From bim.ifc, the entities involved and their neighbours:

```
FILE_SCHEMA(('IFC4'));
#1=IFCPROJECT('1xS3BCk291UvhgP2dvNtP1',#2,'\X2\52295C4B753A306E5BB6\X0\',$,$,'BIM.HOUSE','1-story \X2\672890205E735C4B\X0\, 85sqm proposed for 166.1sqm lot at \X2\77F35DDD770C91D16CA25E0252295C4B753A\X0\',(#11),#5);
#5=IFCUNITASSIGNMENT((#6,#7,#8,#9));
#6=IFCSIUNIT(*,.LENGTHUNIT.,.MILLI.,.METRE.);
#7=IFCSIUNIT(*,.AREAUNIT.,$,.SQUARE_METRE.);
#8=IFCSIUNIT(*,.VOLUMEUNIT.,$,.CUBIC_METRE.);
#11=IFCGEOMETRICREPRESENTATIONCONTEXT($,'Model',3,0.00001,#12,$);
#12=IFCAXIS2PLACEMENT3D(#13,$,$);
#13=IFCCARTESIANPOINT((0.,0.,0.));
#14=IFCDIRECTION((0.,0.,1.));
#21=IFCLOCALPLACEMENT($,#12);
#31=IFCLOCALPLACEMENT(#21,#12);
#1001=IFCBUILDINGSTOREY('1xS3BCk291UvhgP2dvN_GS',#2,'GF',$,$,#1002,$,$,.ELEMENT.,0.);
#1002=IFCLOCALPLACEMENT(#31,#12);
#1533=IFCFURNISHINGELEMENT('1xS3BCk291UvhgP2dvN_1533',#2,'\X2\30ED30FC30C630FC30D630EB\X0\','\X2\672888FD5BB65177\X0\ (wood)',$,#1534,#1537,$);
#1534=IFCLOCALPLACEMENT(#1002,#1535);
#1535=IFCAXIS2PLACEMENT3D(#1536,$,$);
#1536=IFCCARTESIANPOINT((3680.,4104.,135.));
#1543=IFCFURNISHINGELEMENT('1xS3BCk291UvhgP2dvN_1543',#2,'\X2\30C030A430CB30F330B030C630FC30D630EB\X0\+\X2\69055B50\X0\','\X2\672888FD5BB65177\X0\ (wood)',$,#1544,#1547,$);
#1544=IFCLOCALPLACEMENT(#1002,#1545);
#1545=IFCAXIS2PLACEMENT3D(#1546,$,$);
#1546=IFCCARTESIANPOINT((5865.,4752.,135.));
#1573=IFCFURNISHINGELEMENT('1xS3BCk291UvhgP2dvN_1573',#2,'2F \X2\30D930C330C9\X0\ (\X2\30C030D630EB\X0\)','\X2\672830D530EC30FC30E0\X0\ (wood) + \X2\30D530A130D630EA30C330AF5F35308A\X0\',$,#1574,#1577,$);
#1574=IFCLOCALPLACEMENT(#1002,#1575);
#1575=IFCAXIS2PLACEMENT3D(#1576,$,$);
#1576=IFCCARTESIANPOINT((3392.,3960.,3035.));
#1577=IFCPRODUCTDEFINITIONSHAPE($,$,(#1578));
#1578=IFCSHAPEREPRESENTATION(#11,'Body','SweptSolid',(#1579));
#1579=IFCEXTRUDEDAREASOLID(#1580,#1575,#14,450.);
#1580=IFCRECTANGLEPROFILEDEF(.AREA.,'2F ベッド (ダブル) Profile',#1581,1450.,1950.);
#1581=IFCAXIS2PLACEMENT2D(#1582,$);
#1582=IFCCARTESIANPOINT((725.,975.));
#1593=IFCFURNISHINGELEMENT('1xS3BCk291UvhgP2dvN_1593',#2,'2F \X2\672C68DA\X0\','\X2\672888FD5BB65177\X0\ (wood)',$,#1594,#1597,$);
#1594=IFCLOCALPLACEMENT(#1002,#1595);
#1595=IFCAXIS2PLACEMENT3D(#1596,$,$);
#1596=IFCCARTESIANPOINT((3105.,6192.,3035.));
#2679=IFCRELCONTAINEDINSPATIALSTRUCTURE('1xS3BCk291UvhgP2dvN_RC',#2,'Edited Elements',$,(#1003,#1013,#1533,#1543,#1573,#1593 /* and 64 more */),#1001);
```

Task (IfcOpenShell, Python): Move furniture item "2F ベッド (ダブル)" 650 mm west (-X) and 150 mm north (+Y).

```python
import ifcopenshell
import ifcopenshell.api.geometry
import ifcopenshell.util.placement
import ifcopenshell.util.unit

model = ifcopenshell.open("bim.ifc")
unit_scale = ifcopenshell.util.unit.calculate_unit_scale(model)

item = model.by_guid("1xS3BCk291UvhgP2dvN_1573")
matrix = ifcopenshell.util.placement.get_local_placement(item.ObjectPlacement)
matrix[0, 3] -= 0.65 / unit_scale
matrix[1, 3] += 0.15 / unit_scale
ifcopenshell.api.geometry.edit_object_placement(model, product=item, matrix=matrix, is_si=False)

print(ifcopenshell.util.placement.get_local_placement(item.ObjectPlacement).round(3) + 0.0)

model.write("bim_rev.ifc")
```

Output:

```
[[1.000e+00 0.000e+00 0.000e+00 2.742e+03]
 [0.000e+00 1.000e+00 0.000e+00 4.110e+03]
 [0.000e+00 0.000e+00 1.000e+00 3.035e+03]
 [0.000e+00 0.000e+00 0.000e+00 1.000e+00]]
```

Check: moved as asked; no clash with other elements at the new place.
